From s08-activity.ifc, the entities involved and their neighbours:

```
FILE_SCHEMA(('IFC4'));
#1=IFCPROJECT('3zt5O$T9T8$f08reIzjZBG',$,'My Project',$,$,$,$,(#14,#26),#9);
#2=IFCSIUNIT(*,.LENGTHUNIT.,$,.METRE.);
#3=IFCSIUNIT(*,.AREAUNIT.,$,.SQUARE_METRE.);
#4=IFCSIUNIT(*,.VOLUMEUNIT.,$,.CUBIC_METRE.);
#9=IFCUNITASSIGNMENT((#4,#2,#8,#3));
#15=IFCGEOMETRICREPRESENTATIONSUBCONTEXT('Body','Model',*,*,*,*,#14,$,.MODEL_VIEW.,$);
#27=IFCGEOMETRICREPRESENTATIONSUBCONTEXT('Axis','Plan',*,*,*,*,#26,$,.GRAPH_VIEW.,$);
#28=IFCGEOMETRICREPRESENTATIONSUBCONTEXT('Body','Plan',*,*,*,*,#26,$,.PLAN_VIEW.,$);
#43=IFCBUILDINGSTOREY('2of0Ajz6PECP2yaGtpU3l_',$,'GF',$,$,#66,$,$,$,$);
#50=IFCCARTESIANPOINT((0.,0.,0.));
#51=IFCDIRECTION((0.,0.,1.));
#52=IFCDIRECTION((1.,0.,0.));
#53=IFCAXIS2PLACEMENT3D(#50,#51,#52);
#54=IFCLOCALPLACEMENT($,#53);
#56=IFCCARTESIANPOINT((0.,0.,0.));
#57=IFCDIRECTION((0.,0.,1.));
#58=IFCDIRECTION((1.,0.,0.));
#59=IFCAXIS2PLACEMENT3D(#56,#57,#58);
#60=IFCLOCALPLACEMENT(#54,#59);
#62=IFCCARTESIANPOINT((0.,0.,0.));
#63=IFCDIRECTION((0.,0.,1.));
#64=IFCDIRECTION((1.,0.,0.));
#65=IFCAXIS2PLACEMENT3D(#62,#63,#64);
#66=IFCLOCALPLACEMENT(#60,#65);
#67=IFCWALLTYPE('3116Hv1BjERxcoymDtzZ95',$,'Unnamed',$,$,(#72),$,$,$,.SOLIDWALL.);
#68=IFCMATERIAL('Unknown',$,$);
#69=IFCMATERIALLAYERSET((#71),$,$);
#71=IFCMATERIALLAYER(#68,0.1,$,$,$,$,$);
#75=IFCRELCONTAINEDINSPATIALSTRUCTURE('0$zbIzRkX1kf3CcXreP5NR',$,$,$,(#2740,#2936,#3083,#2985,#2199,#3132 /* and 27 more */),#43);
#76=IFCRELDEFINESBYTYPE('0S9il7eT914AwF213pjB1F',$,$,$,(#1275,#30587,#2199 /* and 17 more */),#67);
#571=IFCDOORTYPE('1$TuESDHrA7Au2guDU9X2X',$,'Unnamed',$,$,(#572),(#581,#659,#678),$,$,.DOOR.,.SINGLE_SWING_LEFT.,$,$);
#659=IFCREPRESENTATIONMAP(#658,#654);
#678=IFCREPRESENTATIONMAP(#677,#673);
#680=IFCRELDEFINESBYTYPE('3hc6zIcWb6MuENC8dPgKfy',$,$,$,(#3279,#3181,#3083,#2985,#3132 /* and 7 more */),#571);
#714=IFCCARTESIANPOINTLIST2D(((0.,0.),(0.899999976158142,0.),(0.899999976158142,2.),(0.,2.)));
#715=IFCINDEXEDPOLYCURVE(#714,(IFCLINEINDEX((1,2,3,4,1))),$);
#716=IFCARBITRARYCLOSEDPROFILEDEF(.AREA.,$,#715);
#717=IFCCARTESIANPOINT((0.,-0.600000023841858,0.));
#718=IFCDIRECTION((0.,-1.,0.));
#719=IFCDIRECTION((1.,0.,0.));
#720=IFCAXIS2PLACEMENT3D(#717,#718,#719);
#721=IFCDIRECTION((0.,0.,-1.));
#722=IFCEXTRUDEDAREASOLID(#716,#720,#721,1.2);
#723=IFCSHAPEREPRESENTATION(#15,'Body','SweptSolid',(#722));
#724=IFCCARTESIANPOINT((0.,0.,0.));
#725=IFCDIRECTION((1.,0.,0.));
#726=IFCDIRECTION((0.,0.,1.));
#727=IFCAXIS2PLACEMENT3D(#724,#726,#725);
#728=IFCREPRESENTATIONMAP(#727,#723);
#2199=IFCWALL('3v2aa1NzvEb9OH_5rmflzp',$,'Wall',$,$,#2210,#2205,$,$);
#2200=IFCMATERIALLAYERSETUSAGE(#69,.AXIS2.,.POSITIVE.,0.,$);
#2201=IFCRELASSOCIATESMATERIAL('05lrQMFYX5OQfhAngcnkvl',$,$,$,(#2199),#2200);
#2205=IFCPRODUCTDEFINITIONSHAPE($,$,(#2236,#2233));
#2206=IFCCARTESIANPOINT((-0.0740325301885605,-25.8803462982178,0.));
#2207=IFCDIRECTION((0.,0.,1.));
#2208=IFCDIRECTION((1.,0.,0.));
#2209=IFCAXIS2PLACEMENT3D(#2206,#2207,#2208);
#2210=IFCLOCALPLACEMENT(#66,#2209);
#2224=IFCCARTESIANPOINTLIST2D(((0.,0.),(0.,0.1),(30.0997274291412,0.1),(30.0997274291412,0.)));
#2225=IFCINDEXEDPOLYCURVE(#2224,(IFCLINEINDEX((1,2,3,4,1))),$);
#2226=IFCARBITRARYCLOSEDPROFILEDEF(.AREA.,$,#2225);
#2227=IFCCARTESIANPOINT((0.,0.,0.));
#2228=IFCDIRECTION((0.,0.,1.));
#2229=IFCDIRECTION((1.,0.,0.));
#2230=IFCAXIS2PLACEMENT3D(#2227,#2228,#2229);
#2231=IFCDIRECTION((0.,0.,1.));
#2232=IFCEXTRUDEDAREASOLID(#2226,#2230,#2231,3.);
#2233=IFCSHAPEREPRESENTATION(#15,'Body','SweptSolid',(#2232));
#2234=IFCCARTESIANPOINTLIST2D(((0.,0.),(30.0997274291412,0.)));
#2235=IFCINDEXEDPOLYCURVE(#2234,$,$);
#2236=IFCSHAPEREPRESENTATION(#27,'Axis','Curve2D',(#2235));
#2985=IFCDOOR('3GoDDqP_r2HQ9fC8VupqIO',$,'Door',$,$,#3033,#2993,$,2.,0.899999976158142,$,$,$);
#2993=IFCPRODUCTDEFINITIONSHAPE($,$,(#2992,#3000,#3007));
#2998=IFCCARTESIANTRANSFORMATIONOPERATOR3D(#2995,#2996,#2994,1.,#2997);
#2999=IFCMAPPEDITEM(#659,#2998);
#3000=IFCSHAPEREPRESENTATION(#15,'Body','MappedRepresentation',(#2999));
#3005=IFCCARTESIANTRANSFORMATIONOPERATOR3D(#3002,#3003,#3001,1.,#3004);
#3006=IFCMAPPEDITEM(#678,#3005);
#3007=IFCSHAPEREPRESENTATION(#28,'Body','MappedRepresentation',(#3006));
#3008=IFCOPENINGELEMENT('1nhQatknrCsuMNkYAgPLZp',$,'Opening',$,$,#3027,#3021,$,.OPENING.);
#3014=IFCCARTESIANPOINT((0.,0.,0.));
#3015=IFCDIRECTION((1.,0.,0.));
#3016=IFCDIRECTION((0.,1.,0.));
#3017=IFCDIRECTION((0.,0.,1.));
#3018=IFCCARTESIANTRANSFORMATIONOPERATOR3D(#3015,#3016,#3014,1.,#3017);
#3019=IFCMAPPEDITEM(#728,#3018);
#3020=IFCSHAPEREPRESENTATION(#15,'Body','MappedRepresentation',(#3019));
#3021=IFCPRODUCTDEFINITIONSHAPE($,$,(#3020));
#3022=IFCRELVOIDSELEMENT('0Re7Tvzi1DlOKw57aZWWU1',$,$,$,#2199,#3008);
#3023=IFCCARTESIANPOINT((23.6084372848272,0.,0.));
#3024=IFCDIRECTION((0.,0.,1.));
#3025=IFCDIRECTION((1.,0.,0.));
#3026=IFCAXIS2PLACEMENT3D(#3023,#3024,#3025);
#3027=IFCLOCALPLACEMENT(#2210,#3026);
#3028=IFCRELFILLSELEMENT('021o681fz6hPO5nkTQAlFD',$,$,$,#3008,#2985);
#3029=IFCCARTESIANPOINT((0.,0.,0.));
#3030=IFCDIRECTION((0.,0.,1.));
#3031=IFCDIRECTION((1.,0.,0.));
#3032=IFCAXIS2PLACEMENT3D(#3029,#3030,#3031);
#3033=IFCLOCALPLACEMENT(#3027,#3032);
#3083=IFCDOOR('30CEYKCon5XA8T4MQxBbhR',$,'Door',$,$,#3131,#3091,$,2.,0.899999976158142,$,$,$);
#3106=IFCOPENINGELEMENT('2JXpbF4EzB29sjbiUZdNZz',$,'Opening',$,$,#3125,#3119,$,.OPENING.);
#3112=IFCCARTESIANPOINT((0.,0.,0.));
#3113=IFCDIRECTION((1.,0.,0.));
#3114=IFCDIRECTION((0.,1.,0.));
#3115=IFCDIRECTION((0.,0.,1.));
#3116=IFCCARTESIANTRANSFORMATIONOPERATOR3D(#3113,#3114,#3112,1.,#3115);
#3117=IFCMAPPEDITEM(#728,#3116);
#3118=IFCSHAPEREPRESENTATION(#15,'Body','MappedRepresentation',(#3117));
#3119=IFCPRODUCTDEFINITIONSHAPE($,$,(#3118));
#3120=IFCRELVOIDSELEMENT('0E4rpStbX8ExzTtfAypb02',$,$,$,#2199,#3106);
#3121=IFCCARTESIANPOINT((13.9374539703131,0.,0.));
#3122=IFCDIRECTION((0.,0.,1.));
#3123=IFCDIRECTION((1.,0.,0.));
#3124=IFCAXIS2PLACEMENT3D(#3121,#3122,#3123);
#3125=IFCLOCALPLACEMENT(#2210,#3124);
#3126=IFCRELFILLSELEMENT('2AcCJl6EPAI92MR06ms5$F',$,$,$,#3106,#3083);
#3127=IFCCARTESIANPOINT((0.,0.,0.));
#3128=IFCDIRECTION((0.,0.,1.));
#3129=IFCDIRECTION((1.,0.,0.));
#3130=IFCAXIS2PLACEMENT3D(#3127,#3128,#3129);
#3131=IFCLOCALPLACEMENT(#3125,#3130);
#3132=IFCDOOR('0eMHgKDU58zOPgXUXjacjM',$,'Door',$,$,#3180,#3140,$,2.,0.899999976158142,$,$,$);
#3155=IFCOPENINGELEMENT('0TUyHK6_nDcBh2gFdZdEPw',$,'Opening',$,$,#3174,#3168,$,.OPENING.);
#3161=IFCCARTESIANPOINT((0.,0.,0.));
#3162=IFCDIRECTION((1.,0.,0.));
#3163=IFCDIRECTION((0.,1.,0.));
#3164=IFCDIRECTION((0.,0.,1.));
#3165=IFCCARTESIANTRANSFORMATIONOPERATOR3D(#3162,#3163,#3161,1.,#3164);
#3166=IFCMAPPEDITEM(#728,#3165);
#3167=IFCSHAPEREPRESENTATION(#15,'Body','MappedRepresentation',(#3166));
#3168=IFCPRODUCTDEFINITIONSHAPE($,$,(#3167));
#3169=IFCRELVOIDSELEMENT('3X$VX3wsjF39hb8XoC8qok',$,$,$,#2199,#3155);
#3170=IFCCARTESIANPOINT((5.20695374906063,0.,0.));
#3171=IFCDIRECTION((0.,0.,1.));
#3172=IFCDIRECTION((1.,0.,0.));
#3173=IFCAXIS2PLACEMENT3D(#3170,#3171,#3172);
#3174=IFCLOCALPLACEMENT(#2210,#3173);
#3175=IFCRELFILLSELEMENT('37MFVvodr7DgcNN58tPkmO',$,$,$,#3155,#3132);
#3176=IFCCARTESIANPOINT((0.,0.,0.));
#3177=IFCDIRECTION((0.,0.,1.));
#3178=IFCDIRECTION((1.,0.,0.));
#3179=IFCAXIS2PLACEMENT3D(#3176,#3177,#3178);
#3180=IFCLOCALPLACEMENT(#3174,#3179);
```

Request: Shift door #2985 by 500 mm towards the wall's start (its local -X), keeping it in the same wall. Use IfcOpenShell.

```python
import ifcopenshell
import ifcopenshell.api.geometry
import ifcopenshell.util.placement

model = ifcopenshell.open("s08-activity.ifc")

door = model.by_guid("3GoDDqP_r2HQ9fC8VupqIO")
opening = door.FillsVoids[0].RelatingOpeningElement
wall = opening.VoidsElements[0].RelatingBuildingElement

wall_matrix = ifcopenshell.util.placement.get_local_placement(wall.ObjectPlacement)
shift = wall_matrix[:3, 0] * -0.5
before = ifcopenshell.util.placement.get_local_placement(door.ObjectPlacement)[:3, 3].copy()

# The door is placed relative to its opening, so it follows when the opening moves.
matrix = ifcopenshell.util.placement.get_local_placement(opening.ObjectPlacement)
matrix[:3, 3] += shift
ifcopenshell.api.geometry.edit_object_placement(
    model, product=opening, matrix=matrix, is_si=False, should_transform_children=True
)

after = ifcopenshell.util.placement.get_local_placement(door.ObjectPlacement)[:3, 3]
print("door moved by", (after - before).round(3) + 0.0)

model.write("s08-activity_updated.ifc")
```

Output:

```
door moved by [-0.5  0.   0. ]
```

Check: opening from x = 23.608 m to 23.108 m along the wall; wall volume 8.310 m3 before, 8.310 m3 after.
